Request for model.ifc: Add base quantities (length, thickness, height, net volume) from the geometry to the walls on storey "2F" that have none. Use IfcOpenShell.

First a look at what the model holds.

```python
import ifcopenshell
import ifcopenshell.util.element
import ifcopenshell.util.unit

model = ifcopenshell.open("model.ifc")
print(model.schema)
for unit_type in ("LENGTHUNIT", "AREAUNIT", "VOLUMEUNIT"):
    print(unit_type, ifcopenshell.util.unit.calculate_unit_scale(model, unit_type))
storey = next(s for s in model.by_type("IfcBuildingStorey") if s.Name == "2F")
walls = [e for e in ifcopenshell.util.element.get_decomposition(storey) if e.is_a("IfcWall")]
for e in sorted(walls, key=lambda e: e.id()):
    print(e.id(), e.is_a(), e.Name, list(ifcopenshell.util.element.get_psets(e, qtos_only=True)), sep=" | ")
```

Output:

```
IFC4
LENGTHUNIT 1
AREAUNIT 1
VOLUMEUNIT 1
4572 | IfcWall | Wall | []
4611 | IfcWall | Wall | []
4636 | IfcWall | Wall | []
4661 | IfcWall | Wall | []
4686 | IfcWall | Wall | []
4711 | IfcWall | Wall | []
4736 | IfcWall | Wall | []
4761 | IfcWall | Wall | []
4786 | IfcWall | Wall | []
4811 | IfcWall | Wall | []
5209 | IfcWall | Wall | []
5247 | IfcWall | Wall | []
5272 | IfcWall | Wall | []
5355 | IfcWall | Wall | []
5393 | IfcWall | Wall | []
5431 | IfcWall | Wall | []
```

```python
import ifcopenshell
import ifcopenshell.api.pset
import ifcopenshell.geom
import ifcopenshell.util.element
import ifcopenshell.util.shape
import ifcopenshell.util.unit

model = ifcopenshell.open("model.ifc")
unit_scale = ifcopenshell.util.unit.calculate_unit_scale(model)
volume_scale = ifcopenshell.util.unit.calculate_unit_scale(model, "VOLUMEUNIT")
settings = ifcopenshell.geom.settings()

storey = next(s for s in model.by_type("IfcBuildingStorey") if s.Name == "2F")
walls = [e for e in ifcopenshell.util.element.get_decomposition(storey) if e.is_a("IfcWall")]

for e in sorted(walls, key=lambda e: e.id()):
    if ifcopenshell.util.element.get_psets(e, qtos_only=True, should_inherit=False):
        continue
    # Geometry comes back in metres, in the element's own axes.
    shape = ifcopenshell.geom.create_shape(settings, e)
    values = {
        "Length": ifcopenshell.util.shape.get_x(shape.geometry) / unit_scale,
        "Width": ifcopenshell.util.shape.get_y(shape.geometry) / unit_scale,
        "Height": ifcopenshell.util.shape.get_z(shape.geometry) / unit_scale,
        "NetVolume": ifcopenshell.util.shape.get_volume(shape.geometry) / volume_scale,
    }
    qto = ifcopenshell.api.pset.add_qto(model, product=e, name="Qto_WallBaseQuantities")
    ifcopenshell.api.pset.edit_qto(model, qto=qto, properties=values)
    print(e.id(), {k: round(v, 3) for k, v in values.items()})

model.write("model_edited.ifc")
```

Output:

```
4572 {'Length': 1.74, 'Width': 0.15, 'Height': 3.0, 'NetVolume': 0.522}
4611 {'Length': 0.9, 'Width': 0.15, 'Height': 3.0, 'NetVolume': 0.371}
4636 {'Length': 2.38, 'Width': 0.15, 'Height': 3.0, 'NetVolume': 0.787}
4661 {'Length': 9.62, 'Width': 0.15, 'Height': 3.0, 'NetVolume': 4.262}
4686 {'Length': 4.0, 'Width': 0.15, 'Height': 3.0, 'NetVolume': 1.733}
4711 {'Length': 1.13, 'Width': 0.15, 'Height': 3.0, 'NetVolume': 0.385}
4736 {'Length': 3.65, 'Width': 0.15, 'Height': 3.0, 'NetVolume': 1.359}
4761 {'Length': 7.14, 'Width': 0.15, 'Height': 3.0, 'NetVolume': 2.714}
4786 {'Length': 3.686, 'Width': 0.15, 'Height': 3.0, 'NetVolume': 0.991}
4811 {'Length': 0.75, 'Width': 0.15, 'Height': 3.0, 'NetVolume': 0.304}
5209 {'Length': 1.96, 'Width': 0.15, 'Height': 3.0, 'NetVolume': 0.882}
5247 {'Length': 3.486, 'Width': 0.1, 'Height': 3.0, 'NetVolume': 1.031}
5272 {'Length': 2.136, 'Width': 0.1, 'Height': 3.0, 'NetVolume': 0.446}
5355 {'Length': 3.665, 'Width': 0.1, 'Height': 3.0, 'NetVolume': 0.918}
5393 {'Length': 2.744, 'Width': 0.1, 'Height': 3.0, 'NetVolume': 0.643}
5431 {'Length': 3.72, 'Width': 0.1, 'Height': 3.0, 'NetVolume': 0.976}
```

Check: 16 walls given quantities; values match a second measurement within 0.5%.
